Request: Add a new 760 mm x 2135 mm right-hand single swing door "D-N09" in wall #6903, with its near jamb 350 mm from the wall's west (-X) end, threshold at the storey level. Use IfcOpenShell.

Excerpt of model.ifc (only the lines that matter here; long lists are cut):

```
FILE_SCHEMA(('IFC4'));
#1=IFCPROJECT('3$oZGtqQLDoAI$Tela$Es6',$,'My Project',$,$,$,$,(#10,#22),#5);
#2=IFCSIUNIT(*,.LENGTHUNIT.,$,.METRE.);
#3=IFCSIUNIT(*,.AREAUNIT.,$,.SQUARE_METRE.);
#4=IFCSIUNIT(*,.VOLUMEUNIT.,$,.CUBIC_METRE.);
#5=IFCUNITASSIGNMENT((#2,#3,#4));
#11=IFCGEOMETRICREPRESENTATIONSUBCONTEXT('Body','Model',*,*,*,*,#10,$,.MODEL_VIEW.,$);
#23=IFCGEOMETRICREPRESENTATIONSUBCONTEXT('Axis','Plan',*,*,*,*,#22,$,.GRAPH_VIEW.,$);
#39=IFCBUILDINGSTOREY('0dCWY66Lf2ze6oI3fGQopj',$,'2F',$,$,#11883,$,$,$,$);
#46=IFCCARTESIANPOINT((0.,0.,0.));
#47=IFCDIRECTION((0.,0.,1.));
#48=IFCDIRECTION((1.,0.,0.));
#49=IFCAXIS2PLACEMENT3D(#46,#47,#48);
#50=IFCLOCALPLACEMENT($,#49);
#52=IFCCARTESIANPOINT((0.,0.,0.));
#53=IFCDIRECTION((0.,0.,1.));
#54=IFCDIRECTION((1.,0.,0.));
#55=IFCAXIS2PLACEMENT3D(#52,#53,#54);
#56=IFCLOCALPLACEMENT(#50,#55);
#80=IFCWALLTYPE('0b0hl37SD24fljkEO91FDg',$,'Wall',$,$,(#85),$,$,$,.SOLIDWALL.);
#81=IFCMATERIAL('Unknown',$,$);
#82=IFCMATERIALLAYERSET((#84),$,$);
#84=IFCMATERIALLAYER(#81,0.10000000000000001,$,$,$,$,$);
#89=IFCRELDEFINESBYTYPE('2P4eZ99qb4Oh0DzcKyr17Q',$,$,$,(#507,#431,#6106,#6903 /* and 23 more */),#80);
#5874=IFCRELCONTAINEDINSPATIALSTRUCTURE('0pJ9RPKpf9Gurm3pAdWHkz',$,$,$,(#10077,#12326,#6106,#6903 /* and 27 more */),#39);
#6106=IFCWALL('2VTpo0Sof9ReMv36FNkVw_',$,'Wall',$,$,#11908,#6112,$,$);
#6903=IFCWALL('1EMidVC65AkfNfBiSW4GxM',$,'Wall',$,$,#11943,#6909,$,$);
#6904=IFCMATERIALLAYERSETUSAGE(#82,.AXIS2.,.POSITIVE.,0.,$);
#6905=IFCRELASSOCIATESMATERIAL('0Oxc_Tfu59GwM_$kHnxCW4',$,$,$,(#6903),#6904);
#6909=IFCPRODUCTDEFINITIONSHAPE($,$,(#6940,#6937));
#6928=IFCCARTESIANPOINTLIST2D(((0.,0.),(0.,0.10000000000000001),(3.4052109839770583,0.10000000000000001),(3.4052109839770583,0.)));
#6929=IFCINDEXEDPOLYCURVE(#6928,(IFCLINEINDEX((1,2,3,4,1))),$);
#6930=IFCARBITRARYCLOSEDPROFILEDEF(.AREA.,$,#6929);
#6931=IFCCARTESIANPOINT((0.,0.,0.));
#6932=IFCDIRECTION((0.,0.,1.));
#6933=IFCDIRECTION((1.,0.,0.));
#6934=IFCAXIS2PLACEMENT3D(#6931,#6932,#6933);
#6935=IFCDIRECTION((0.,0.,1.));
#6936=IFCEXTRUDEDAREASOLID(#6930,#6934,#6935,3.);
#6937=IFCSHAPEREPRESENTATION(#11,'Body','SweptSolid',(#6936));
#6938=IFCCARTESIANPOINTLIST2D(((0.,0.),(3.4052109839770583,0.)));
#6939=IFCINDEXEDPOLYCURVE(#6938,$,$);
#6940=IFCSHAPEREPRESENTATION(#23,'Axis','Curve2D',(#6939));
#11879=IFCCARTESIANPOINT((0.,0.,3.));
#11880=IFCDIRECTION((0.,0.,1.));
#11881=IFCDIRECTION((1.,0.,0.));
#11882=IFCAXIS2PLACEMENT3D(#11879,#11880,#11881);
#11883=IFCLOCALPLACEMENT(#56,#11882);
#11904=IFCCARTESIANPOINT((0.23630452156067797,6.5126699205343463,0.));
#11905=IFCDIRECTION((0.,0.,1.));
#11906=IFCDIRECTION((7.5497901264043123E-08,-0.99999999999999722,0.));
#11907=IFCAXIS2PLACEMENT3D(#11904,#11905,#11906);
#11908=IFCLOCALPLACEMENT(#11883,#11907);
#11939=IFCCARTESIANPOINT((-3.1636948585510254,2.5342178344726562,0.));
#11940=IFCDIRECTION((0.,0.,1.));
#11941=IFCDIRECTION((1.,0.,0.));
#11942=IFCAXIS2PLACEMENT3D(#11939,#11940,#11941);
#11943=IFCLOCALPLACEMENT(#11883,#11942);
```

```python
import numpy as np
import ifcopenshell
import ifcopenshell.api.feature
import ifcopenshell.api.geometry
import ifcopenshell.api.root
import ifcopenshell.api.spatial
import ifcopenshell.geom
import ifcopenshell.util.element
import ifcopenshell.util.placement
import ifcopenshell.util.representation
import ifcopenshell.util.shape
import ifcopenshell.util.unit

model = ifcopenshell.open("model.ifc")
unit_scale = ifcopenshell.util.unit.calculate_unit_scale(model)
settings = ifcopenshell.geom.settings()


def volume(element):
    """Net volume in cubic metres, openings subtracted."""
    shape = ifcopenshell.geom.create_shape(settings, element)
    return ifcopenshell.util.shape.get_volume(shape.geometry)


wall = model.by_guid("1EMidVC65AkfNfBiSW4GxM")
storey = ifcopenshell.util.element.get_container(wall, ifc_class="IfcBuildingStorey")
context = ifcopenshell.util.representation.get_context(model, "Model", "Body", "MODEL_VIEW")
before = volume(wall)

width, height, from_end, sill = 0.76, 2.135, 0.35, 0.0  # metres

# The wall runs along its own X axis, and the end named is its -X end.
wall_shape = ifcopenshell.geom.create_shape(settings, wall)
x, y, z = ifcopenshell.util.shape.get_vertices(wall_shape.geometry).T
start = x.min() + from_end
face, thickness = float(y.min()), float(y.max() - y.min())
wall_matrix = ifcopenshell.util.placement.get_local_placement(wall.ObjectPlacement)
level = ifcopenshell.util.placement.get_local_placement(storey.ObjectPlacement)[2, 3]


def in_wall(x, y):
    """Placement at x, y metres in the wall's axes, at sill height."""
    matrix = wall_matrix.copy()
    matrix[:, 3] = wall_matrix @ np.array([x / unit_scale, y / unit_scale, 0.0, 1.0])
    matrix[2, 3] = level + sill / unit_scale
    return matrix


# Opening: a box that overshoots both wall faces by 50 mm.
opening = ifcopenshell.api.root.create_entity(model, ifc_class="IfcOpeningElement", predefined_type="OPENING")
box = ifcopenshell.api.geometry.add_wall_representation(
    model, context=context, length=width, height=height, thickness=thickness + 0.1
)
ifcopenshell.api.geometry.assign_representation(model, product=opening, representation=box)
ifcopenshell.api.geometry.edit_object_placement(model, product=opening, matrix=in_wall(start, face - 0.05), is_si=False)
ifcopenshell.api.feature.add_feature(model, feature=opening, element=wall)

door = ifcopenshell.api.root.create_entity(model, ifc_class="IfcDoor", name="D-N09", predefined_type="DOOR")
door.OverallWidth, door.OverallHeight = width / unit_scale, height / unit_scale
door.OperationType = "SINGLE_SWING_RIGHT"
body = ifcopenshell.api.geometry.add_door_representation(
    model,
    context=context,
    overall_width=door.OverallWidth,
    overall_height=door.OverallHeight,
    operation_type="SINGLE_SWING_RIGHT",
    lining_properties={"LiningDepth": thickness / unit_scale, "ThresholdDepth": thickness / unit_scale},
)
ifcopenshell.api.geometry.assign_representation(model, product=door, representation=body)
ifcopenshell.api.spatial.assign_container(model, products=[door], relating_structure=storey)
ifcopenshell.api.feature.add_filling(model, opening=opening, element=door)

# The lining spans the wall, so the door starts at the wall face.
ifcopenshell.api.geometry.edit_object_placement(model, product=door, matrix=in_wall(start, face), is_si=False)

after = volume(wall)

print(f"wall volume {before:.3f} -> {after:.3f} m3")

model.write("model_rev.ifc")
```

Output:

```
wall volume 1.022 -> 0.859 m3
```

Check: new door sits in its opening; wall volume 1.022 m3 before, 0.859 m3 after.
